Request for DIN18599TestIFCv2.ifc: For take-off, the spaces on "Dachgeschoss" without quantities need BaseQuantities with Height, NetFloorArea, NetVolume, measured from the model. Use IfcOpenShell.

First a look at what the model holds.

```python
import ifcopenshell
import ifcopenshell.util.element
import ifcopenshell.util.unit

model = ifcopenshell.open("DIN18599TestIFCv2.ifc")
print(model.schema)
for unit_type in ("LENGTHUNIT", "AREAUNIT", "VOLUMEUNIT"):
    print(unit_type, ifcopenshell.util.unit.calculate_unit_scale(model, unit_type))
storey = next(s for s in model.by_type("IfcBuildingStorey") if s.Name == "Dachgeschoss")
spaces = [e for e in ifcopenshell.util.element.get_decomposition(storey) if e.is_a("IfcSpace")]
for e in sorted(spaces, key=lambda e: e.id()):
    print(e.id(), e.is_a(), e.Name, list(ifcopenshell.util.element.get_psets(e, qtos_only=True)), sep=" | ")
```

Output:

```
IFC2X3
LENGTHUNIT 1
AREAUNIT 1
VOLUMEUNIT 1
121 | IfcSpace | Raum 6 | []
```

```python
import ifcopenshell
import ifcopenshell.api.pset
import ifcopenshell.geom
import ifcopenshell.util.element
import ifcopenshell.util.shape
import ifcopenshell.util.unit

model = ifcopenshell.open("DIN18599TestIFCv2.ifc")
unit_scale = ifcopenshell.util.unit.calculate_unit_scale(model)
area_scale = ifcopenshell.util.unit.calculate_unit_scale(model, "AREAUNIT")
volume_scale = ifcopenshell.util.unit.calculate_unit_scale(model, "VOLUMEUNIT")
settings = ifcopenshell.geom.settings()

storey = next(s for s in model.by_type("IfcBuildingStorey") if s.Name == "Dachgeschoss")
spaces = [e for e in ifcopenshell.util.element.get_decomposition(storey) if e.is_a("IfcSpace")]

for e in sorted(spaces, key=lambda e: e.id()):
    if ifcopenshell.util.element.get_psets(e, qtos_only=True, should_inherit=False):
        continue
    # Geometry comes back in metres, in the element's own axes.
    shape = ifcopenshell.geom.create_shape(settings, e)
    values = {
        "Height": ifcopenshell.util.shape.get_z(shape.geometry) / unit_scale,
        "NetFloorArea": ifcopenshell.util.shape.get_footprint_area(shape.geometry) / area_scale,
        "NetVolume": ifcopenshell.util.shape.get_volume(shape.geometry) / volume_scale,
    }
    qto = ifcopenshell.api.pset.add_qto(model, product=e, name="BaseQuantities")
    ifcopenshell.api.pset.edit_qto(model, qto=qto, properties=values)
    print(e.id(), {k: round(v, 3) for k, v in values.items()})

model.write("DIN18599TestIFCv2_edited.ifc")
```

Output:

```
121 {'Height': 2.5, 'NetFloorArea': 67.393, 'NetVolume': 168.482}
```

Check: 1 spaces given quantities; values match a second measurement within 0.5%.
